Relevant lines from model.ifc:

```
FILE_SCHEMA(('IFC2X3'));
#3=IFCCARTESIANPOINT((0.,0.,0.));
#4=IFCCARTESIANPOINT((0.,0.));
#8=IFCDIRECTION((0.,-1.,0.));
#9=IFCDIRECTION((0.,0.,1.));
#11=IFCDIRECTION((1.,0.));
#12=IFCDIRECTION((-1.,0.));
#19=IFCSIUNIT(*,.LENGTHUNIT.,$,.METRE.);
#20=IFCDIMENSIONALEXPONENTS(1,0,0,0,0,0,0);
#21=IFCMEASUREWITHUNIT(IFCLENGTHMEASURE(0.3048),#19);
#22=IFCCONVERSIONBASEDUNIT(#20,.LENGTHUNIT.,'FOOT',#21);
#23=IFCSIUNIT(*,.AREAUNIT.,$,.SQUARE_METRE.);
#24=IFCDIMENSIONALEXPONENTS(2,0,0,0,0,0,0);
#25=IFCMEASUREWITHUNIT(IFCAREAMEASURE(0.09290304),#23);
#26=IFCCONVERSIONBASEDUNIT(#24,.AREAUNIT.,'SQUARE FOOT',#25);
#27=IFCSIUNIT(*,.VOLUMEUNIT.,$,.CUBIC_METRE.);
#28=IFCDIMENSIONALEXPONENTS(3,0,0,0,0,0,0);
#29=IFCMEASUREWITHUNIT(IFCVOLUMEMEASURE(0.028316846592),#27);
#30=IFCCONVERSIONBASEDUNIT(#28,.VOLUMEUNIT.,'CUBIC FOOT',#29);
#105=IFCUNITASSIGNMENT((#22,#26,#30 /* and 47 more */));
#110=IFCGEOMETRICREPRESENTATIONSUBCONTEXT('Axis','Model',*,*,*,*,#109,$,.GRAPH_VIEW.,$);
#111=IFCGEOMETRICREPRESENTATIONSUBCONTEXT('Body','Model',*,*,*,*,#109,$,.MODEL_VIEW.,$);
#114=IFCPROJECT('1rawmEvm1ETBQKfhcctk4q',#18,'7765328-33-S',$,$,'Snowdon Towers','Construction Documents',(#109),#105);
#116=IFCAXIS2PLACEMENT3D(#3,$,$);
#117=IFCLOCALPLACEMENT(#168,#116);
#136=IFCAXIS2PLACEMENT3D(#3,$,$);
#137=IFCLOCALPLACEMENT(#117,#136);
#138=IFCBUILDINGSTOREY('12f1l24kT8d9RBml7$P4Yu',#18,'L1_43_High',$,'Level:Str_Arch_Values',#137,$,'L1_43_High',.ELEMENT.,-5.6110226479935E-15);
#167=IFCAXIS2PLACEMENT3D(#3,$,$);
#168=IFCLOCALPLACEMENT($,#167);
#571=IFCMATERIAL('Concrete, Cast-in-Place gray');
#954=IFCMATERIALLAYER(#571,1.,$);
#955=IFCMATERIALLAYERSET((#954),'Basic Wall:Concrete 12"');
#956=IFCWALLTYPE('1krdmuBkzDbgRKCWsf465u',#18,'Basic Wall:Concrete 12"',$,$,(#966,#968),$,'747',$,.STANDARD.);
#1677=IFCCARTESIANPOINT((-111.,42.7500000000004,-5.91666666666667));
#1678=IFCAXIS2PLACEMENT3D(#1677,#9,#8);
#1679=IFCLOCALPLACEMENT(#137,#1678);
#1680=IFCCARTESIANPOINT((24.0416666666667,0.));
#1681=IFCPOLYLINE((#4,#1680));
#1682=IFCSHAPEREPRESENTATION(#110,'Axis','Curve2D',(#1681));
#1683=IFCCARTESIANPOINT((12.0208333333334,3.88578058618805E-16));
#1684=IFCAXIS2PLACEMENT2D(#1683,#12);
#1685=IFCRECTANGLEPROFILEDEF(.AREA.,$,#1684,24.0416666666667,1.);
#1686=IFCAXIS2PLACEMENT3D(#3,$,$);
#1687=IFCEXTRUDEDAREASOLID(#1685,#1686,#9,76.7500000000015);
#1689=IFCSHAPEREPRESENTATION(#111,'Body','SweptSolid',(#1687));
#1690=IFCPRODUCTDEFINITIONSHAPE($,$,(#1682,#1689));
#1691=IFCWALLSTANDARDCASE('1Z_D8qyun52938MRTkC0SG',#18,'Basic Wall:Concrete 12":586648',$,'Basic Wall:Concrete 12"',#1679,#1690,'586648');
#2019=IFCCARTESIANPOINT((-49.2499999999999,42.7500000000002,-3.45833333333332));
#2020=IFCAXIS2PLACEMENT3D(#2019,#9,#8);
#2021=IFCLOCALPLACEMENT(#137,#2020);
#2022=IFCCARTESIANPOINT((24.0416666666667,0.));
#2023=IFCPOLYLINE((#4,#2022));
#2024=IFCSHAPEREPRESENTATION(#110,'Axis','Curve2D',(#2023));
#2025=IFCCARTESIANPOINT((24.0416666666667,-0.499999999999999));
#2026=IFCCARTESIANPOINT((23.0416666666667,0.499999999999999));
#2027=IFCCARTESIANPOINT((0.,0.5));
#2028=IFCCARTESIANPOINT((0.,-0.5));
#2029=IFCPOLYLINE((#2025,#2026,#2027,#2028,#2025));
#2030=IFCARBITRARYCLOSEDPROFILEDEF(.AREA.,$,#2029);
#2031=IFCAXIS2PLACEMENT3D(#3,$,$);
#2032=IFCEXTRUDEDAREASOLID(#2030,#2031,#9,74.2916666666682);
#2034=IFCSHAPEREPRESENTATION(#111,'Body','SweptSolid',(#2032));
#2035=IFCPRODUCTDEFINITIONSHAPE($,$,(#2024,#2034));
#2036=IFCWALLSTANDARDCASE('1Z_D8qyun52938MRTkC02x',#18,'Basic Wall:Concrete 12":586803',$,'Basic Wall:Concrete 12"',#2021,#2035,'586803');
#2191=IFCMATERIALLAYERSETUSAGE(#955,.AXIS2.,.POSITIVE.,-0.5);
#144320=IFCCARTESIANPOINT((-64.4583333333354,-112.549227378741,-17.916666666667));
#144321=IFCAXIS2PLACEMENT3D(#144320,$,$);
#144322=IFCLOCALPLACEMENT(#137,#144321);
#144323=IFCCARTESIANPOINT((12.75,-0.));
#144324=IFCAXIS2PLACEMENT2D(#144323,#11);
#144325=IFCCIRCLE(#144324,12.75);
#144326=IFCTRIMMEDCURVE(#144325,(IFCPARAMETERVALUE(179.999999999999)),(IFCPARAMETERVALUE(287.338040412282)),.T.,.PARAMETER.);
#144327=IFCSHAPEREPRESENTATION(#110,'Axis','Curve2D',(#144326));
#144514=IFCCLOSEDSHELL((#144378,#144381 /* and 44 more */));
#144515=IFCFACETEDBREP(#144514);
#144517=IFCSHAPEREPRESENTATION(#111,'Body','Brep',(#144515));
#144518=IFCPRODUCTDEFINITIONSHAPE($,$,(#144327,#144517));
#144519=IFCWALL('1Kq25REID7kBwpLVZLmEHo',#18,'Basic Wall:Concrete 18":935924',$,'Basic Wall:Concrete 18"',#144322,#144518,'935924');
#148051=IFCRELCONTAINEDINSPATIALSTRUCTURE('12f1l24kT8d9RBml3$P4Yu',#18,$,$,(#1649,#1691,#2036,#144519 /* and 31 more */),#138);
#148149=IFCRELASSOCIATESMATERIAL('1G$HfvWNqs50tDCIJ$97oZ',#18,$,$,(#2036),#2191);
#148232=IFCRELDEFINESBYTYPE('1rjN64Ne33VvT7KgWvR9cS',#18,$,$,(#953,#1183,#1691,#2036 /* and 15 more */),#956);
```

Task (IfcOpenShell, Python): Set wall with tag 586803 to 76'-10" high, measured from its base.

```python
import ifcopenshell
import ifcopenshell.geom
import ifcopenshell.util.representation
import ifcopenshell.util.shape
import ifcopenshell.util.unit

model = ifcopenshell.open("model.ifc")
unit_scale = ifcopenshell.util.unit.calculate_unit_scale(model)
settings = ifcopenshell.geom.settings()


def volume(element):
    """Net volume in cubic metres, openings subtracted."""
    shape = ifcopenshell.geom.create_shape(settings, element)
    return ifcopenshell.util.shape.get_volume(shape.geometry)


wall = model.by_id(2036)
before = volume(wall)

body = ifcopenshell.util.representation.get_representation(wall, "Model", "Body")
solid = body.Items[0]
old_height = solid.Depth
solid.Depth = 922 * 0.0254 / unit_scale
after = volume(wall)

print(f"height {old_height:g} -> {solid.Depth:g}, volume {before:.3f} -> {after:.3f} m3")

model.write("model_updated.ifc")
```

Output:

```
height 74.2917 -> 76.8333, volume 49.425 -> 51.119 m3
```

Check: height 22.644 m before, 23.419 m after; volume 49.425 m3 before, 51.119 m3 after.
